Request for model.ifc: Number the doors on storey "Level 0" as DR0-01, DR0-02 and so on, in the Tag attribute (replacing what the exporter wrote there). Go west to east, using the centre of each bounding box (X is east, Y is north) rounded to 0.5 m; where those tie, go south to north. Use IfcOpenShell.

First a look at what the model holds.

```python
import ifcopenshell
import ifcopenshell.util.element
import ifcopenshell.util.placement

model = ifcopenshell.open("model.ifc")
print(model.schema)
storey = next(s for s in model.by_type("IfcBuildingStorey") if s.Name == "Level 0")
doors = [e for e in ifcopenshell.util.element.get_decomposition(storey) if e.is_a("IfcDoor")]
for e in sorted(doors, key=lambda e: e.id()):
    origin = ifcopenshell.util.placement.get_local_placement(e.ObjectPlacement)[:3, 3]
    print(e.id(), e.Tag, e.Name, origin.round(2) + 0.0, sep=" | ")
```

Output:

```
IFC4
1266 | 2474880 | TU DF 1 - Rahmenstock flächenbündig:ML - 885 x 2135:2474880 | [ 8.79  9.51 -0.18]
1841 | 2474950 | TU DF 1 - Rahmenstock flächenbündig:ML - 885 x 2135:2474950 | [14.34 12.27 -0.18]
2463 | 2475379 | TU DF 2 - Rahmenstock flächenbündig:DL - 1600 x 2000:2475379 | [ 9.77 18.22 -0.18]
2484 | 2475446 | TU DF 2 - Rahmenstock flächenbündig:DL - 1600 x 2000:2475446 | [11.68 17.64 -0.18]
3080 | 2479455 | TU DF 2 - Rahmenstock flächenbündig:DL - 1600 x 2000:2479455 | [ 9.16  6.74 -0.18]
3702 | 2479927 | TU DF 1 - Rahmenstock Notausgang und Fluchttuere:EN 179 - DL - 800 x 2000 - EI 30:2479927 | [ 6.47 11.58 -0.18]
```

```python
import ifcopenshell
import ifcopenshell.geom
import ifcopenshell.util.element
import ifcopenshell.util.shape

model = ifcopenshell.open("model.ifc")
settings = ifcopenshell.geom.settings()
settings.set("use-world-coords", True)


def centre(element):
    shape = ifcopenshell.geom.create_shape(settings, element)
    return ifcopenshell.util.shape.get_bbox_centroid(shape.geometry)


storey = next(s for s in model.by_type("IfcBuildingStorey") if s.Name == "Level 0")
doors = [e for e in ifcopenshell.util.element.get_decomposition(storey) if e.is_a("IfcDoor")]

# Insertion points can sit at a corner or the storey origin, so sort by the geometry (in metres).
centres = {e: centre(e) for e in doors}
doors.sort(key=lambda e: (round(centres[e][0] / 0.5), centres[e][1]))

for i, e in enumerate(doors, start=1):
    number = f"DR0-{i:02d}"
    e.Tag = number
    print(e.id(), number)

model.write("model_edited.ifc")
```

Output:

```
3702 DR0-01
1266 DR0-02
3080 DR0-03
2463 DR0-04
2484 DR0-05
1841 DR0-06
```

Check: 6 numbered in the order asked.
